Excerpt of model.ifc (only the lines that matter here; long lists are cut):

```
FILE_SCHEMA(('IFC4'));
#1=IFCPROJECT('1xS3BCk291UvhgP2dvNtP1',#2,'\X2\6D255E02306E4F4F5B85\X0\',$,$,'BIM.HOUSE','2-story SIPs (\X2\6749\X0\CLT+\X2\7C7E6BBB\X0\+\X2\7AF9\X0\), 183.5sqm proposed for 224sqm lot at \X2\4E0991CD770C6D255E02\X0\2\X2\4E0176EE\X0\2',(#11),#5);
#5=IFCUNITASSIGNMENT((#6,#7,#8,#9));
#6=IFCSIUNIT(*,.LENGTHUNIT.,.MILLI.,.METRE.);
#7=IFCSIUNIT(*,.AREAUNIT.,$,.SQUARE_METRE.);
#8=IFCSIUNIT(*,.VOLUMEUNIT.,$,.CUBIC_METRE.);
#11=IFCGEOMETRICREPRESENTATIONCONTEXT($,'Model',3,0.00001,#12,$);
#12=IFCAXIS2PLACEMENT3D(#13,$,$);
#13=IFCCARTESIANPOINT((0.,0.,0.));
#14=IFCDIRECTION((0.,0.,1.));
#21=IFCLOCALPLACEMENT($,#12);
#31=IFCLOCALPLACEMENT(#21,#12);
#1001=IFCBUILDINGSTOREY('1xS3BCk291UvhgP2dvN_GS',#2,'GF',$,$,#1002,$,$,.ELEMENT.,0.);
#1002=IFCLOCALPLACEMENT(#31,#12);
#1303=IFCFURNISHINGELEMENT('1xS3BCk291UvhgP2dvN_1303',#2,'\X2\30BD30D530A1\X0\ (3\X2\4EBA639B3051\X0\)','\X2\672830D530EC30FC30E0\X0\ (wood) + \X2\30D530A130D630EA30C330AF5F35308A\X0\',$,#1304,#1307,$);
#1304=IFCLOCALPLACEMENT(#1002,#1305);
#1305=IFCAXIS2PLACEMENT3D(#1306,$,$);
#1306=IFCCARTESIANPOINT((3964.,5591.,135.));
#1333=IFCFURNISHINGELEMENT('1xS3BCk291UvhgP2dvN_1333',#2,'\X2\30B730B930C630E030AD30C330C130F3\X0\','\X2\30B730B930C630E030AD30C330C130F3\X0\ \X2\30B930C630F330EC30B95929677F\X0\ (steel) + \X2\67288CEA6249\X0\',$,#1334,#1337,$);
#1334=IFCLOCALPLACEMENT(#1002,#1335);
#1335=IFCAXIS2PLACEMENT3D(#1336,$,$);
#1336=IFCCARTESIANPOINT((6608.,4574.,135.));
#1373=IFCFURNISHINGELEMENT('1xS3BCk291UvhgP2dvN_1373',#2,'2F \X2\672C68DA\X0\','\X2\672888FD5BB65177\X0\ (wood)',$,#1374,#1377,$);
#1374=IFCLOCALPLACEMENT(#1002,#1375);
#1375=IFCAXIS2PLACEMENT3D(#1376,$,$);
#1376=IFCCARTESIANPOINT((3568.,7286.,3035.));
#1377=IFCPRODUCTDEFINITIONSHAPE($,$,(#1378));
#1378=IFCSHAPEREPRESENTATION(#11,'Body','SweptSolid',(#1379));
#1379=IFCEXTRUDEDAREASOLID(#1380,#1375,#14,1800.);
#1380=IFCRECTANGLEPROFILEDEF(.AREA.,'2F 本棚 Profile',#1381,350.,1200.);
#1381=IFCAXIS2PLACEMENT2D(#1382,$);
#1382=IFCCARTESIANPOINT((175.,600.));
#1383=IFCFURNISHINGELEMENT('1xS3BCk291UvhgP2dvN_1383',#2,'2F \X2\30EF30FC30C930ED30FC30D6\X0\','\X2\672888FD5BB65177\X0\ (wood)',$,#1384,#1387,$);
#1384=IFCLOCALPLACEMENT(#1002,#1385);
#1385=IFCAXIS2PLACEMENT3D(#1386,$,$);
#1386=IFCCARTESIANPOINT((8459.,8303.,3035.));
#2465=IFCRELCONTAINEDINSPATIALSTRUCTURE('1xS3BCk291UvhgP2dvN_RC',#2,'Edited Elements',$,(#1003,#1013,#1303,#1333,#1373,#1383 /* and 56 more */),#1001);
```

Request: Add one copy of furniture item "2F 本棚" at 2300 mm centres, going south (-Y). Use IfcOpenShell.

```python
import numpy as np
import ifcopenshell
import ifcopenshell.api.geometry
import ifcopenshell.api.root
import ifcopenshell.util.element
import ifcopenshell.util.placement

model = ifcopenshell.open("model.ifc")


def reuse_history(source, copy):
    """copy_class also copies each property set's owner history, people and application; keep the originals."""
    for rel in copy.IsDefinedBy:
        if rel.is_a("IfcRelDefinesByProperties") and (history := rel.RelatingPropertyDefinition.OwnerHistory):
            rel.RelatingPropertyDefinition.OwnerHistory = source.OwnerHistory
            ifcopenshell.util.element.remove_deep2(model, history)


source = model.by_id(1373)
base = ifcopenshell.util.placement.get_local_placement(source.ObjectPlacement)
step = np.array([0.0, -1.0, 0.0]) * 2300.0

for i in range(1, 2):
    copy = ifcopenshell.api.root.copy_class(model, product=source)
    copy.Representation = ifcopenshell.util.element.copy_deep(
        model, source.Representation, exclude=["IfcGeometricRepresentationContext", "IfcRepresentationMap"]
    )
    reuse_history(source, copy)
    matrix = base.copy()
    matrix[:3, 3] += i * step
    print("added at", matrix[:3, 3].round(3) + 0.0)
    ifcopenshell.api.geometry.edit_object_placement(model, product=copy, matrix=matrix, is_si=False)

model.write("model_v2.ifc")
```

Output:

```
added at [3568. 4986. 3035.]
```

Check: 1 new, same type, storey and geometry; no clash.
